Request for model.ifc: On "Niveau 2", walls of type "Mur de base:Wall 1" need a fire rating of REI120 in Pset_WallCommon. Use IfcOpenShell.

First a look at what the model holds.

```python
import ifcopenshell
import ifcopenshell.util.element

model = ifcopenshell.open("model.ifc")
print(model.schema)
storey = next(s for s in model.by_type("IfcBuildingStorey") if s.Name == "Niveau 2")
walls = [e for e in ifcopenshell.util.element.get_decomposition(storey) if e.is_a("IfcWall")]
seen = {}
for e in walls:
    element_type = ifcopenshell.util.element.get_type(e)
    key = (element_type.Name if element_type != e and element_type else None, ifcopenshell.util.element.get_pset(e, "Pset_WallCommon", "FireRating"))
    seen[key] = seen.get(key, 0) + 1
for (name, value), count in sorted(seen.items(), key=str):
    print(count, "x", name, "|", value)
```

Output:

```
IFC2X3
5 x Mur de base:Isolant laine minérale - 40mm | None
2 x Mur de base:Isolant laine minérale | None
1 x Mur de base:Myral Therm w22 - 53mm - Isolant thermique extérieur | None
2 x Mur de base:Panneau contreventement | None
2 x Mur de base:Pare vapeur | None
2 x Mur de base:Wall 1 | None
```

```python
import ifcopenshell
import ifcopenshell.api.pset
import ifcopenshell.util.element

model = ifcopenshell.open("model.ifc")

storey = next(s for s in model.by_type("IfcBuildingStorey") if s.Name == "Niveau 2")
walls = [e for e in ifcopenshell.util.element.get_decomposition(storey) if e.is_a("IfcWall")]

count = 0
for e in walls:
    element_type = ifcopenshell.util.element.get_type(e)
    if element_type in (None, e) or element_type.Name != "Mur de base:Wall 1":
        continue
    # add_pset returns the element's existing set when there is one.
    pset = ifcopenshell.api.pset.add_pset(model, product=e, name="Pset_WallCommon")
    ifcopenshell.api.pset.edit_pset(model, pset=pset, properties={"FireRating": "REI120"})
    count += 1

print(count, "walls updated")

model.write("model_rev.ifc")
```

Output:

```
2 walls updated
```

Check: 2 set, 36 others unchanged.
